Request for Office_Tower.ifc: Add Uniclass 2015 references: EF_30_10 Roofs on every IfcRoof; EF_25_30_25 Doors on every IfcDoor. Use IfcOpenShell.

First a look at what the model holds.

```python
import ifcopenshell

model = ifcopenshell.open("Office_Tower.ifc")
print(model.schema)
print("classifications:", [c.Name for c in model.by_type("IfcClassification")])
for ifc_class in ("IfcDoor", "IfcRoof", "IfcStair", "IfcWall", "IfcWindow"):
    print(ifc_class, len(model.by_type(ifc_class)))
```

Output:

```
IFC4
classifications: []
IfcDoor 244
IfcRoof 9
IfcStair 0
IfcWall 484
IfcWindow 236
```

```python
import ifcopenshell
import ifcopenshell.api.classification

model = ifcopenshell.open("Office_Tower.ifc")

system = ifcopenshell.api.classification.add_classification(model, classification="Uniclass 2015")

codes = {
    "IfcRoof": ("EF_30_10", "Roofs"),
    "IfcDoor": ("EF_25_30_25", "Doors"),
}
for ifc_class, (code, name) in codes.items():
    products = model.by_type(ifc_class)
    ifcopenshell.api.classification.add_reference(
        model, products=products, classification=system, identification=code, name=name
    )
    print(code, len(products))

model.write("Office_Tower-out.ifc")
```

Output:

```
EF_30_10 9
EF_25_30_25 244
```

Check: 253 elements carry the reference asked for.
